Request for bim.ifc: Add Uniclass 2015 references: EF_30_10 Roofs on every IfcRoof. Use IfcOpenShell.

First a look at what the model holds.

```python
import ifcopenshell

model = ifcopenshell.open("bim.ifc")
print(model.schema)
print("classifications:", [c.Name for c in model.by_type("IfcClassification")])
for ifc_class in ("IfcDoor", "IfcRoof", "IfcStair", "IfcWall", "IfcWindow"):
    print(ifc_class, len(model.by_type(ifc_class)))
```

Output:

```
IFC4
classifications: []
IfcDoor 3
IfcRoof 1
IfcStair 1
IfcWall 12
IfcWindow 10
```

```python
import ifcopenshell
import ifcopenshell.api.classification

model = ifcopenshell.open("bim.ifc")

system = ifcopenshell.api.classification.add_classification(model, classification="Uniclass 2015")

codes = {
    "IfcRoof": ("EF_30_10", "Roofs"),
}
for ifc_class, (code, name) in codes.items():
    products = model.by_type(ifc_class)
    ifcopenshell.api.classification.add_reference(
        model, products=products, classification=system, identification=code, name=name
    )
    print(code, len(products))

model.write("bim_edited.ifc")
```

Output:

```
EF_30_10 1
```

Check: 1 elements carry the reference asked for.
